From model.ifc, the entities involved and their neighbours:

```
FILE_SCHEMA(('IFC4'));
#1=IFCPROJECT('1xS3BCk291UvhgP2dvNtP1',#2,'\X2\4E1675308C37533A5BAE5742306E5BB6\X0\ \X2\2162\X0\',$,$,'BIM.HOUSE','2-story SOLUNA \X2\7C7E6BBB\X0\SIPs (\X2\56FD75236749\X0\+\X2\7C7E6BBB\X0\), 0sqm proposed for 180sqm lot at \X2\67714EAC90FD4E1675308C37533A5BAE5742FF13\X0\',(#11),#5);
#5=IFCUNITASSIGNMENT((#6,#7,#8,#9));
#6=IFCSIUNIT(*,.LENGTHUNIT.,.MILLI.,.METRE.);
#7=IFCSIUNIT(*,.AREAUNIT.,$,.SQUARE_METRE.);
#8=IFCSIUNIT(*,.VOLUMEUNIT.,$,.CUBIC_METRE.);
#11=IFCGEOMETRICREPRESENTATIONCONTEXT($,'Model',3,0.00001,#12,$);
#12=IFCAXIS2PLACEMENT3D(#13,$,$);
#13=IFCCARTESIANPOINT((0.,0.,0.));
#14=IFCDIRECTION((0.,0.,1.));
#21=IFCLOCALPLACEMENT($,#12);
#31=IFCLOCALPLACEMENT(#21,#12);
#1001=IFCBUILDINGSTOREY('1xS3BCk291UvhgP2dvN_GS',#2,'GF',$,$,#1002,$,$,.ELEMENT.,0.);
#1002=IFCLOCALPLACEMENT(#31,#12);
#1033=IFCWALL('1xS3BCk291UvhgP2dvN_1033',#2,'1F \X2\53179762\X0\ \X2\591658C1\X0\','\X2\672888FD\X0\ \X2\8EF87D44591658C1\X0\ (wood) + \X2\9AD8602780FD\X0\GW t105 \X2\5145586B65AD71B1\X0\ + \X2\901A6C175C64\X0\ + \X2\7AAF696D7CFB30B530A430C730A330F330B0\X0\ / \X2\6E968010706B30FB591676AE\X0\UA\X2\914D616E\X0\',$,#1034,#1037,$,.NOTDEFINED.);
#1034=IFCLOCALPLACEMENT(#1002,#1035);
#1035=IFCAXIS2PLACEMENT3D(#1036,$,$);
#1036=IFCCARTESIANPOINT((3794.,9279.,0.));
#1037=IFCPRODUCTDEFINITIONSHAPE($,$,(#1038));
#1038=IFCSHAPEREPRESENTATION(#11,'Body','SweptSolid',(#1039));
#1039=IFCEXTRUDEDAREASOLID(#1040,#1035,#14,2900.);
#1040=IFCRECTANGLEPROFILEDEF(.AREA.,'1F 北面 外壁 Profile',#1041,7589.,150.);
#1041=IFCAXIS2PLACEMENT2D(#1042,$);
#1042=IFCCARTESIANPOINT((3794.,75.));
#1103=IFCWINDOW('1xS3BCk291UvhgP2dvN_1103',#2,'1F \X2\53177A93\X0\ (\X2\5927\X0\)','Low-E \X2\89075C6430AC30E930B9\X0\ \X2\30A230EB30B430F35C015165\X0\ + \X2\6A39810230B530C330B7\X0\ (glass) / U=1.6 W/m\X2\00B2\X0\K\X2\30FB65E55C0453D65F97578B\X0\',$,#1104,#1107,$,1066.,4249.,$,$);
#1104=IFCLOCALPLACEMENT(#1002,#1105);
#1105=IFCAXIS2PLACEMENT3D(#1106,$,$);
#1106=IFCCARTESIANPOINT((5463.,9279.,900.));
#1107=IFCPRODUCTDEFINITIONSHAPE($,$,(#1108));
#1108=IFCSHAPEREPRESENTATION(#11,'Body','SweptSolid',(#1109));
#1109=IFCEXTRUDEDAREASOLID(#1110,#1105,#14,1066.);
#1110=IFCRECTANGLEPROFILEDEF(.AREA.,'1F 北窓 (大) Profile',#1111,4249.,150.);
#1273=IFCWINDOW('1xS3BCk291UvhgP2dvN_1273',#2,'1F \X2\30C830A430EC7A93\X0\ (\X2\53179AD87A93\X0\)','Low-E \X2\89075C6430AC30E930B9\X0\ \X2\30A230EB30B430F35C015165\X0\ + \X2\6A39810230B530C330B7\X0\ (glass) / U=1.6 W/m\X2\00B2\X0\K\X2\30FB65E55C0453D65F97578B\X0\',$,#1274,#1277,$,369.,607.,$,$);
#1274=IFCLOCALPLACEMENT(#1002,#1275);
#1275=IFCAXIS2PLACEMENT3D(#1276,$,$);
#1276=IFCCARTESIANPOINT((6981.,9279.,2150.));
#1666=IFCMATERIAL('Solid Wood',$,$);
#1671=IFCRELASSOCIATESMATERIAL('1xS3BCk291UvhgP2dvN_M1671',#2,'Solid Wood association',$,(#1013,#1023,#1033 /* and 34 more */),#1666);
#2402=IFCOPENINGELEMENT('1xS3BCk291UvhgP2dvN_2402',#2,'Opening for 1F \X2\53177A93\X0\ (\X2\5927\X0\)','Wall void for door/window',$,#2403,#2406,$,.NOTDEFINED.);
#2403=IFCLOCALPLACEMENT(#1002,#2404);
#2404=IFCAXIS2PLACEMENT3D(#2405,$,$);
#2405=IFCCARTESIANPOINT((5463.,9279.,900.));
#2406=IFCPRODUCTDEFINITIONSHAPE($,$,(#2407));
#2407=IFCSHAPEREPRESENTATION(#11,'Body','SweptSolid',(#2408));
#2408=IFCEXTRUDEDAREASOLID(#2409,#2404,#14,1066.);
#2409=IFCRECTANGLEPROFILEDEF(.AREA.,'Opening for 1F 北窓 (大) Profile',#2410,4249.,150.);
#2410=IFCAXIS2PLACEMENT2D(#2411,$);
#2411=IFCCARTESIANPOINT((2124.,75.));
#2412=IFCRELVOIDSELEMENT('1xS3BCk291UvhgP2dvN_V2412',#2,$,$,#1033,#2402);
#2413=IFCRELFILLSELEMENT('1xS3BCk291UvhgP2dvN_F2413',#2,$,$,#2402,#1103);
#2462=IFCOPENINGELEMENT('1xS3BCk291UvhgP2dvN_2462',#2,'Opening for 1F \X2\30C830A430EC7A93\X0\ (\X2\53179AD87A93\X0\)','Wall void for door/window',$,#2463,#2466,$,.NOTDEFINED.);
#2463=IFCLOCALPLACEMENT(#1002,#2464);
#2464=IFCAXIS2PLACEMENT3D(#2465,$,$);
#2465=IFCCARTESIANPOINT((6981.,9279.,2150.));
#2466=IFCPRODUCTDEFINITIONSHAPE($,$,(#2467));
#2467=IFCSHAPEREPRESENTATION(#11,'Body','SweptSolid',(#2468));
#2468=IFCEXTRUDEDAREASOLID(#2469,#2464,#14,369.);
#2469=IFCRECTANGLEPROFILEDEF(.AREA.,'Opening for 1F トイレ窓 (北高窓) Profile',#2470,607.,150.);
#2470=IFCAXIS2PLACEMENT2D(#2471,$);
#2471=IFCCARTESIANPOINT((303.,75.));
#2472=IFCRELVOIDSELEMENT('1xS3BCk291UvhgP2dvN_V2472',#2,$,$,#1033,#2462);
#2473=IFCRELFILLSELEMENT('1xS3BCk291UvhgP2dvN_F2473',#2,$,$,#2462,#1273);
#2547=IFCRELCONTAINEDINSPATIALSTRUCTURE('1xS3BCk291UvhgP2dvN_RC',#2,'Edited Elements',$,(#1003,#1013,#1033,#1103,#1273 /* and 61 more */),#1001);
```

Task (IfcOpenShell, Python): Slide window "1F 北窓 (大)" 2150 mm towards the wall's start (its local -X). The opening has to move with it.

```python
import ifcopenshell
import ifcopenshell.api.geometry
import ifcopenshell.util.placement
import ifcopenshell.util.unit

model = ifcopenshell.open("model.ifc")
unit_scale = ifcopenshell.util.unit.calculate_unit_scale(model)

window = model.by_guid("1xS3BCk291UvhgP2dvN_1103")
opening = window.FillsVoids[0].RelatingOpeningElement
wall = opening.VoidsElements[0].RelatingBuildingElement

wall_matrix = ifcopenshell.util.placement.get_local_placement(wall.ObjectPlacement)
shift = wall_matrix[:3, 0] * -2.15 / unit_scale
before = ifcopenshell.util.placement.get_local_placement(window.ObjectPlacement)[:3, 3].copy()

# The window is not placed relative to its opening, so move both.
for product in (opening, window):
    matrix = ifcopenshell.util.placement.get_local_placement(product.ObjectPlacement)
    matrix[:3, 3] += shift
    ifcopenshell.api.geometry.edit_object_placement(model, product=product, matrix=matrix, is_si=False)

after = ifcopenshell.util.placement.get_local_placement(window.ObjectPlacement)[:3, 3]
print("window moved by", (after - before).round(3) + 0.0)

model.write("model_v2.ifc")
```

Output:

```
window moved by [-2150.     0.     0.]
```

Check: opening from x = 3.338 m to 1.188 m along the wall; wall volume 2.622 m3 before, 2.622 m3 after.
